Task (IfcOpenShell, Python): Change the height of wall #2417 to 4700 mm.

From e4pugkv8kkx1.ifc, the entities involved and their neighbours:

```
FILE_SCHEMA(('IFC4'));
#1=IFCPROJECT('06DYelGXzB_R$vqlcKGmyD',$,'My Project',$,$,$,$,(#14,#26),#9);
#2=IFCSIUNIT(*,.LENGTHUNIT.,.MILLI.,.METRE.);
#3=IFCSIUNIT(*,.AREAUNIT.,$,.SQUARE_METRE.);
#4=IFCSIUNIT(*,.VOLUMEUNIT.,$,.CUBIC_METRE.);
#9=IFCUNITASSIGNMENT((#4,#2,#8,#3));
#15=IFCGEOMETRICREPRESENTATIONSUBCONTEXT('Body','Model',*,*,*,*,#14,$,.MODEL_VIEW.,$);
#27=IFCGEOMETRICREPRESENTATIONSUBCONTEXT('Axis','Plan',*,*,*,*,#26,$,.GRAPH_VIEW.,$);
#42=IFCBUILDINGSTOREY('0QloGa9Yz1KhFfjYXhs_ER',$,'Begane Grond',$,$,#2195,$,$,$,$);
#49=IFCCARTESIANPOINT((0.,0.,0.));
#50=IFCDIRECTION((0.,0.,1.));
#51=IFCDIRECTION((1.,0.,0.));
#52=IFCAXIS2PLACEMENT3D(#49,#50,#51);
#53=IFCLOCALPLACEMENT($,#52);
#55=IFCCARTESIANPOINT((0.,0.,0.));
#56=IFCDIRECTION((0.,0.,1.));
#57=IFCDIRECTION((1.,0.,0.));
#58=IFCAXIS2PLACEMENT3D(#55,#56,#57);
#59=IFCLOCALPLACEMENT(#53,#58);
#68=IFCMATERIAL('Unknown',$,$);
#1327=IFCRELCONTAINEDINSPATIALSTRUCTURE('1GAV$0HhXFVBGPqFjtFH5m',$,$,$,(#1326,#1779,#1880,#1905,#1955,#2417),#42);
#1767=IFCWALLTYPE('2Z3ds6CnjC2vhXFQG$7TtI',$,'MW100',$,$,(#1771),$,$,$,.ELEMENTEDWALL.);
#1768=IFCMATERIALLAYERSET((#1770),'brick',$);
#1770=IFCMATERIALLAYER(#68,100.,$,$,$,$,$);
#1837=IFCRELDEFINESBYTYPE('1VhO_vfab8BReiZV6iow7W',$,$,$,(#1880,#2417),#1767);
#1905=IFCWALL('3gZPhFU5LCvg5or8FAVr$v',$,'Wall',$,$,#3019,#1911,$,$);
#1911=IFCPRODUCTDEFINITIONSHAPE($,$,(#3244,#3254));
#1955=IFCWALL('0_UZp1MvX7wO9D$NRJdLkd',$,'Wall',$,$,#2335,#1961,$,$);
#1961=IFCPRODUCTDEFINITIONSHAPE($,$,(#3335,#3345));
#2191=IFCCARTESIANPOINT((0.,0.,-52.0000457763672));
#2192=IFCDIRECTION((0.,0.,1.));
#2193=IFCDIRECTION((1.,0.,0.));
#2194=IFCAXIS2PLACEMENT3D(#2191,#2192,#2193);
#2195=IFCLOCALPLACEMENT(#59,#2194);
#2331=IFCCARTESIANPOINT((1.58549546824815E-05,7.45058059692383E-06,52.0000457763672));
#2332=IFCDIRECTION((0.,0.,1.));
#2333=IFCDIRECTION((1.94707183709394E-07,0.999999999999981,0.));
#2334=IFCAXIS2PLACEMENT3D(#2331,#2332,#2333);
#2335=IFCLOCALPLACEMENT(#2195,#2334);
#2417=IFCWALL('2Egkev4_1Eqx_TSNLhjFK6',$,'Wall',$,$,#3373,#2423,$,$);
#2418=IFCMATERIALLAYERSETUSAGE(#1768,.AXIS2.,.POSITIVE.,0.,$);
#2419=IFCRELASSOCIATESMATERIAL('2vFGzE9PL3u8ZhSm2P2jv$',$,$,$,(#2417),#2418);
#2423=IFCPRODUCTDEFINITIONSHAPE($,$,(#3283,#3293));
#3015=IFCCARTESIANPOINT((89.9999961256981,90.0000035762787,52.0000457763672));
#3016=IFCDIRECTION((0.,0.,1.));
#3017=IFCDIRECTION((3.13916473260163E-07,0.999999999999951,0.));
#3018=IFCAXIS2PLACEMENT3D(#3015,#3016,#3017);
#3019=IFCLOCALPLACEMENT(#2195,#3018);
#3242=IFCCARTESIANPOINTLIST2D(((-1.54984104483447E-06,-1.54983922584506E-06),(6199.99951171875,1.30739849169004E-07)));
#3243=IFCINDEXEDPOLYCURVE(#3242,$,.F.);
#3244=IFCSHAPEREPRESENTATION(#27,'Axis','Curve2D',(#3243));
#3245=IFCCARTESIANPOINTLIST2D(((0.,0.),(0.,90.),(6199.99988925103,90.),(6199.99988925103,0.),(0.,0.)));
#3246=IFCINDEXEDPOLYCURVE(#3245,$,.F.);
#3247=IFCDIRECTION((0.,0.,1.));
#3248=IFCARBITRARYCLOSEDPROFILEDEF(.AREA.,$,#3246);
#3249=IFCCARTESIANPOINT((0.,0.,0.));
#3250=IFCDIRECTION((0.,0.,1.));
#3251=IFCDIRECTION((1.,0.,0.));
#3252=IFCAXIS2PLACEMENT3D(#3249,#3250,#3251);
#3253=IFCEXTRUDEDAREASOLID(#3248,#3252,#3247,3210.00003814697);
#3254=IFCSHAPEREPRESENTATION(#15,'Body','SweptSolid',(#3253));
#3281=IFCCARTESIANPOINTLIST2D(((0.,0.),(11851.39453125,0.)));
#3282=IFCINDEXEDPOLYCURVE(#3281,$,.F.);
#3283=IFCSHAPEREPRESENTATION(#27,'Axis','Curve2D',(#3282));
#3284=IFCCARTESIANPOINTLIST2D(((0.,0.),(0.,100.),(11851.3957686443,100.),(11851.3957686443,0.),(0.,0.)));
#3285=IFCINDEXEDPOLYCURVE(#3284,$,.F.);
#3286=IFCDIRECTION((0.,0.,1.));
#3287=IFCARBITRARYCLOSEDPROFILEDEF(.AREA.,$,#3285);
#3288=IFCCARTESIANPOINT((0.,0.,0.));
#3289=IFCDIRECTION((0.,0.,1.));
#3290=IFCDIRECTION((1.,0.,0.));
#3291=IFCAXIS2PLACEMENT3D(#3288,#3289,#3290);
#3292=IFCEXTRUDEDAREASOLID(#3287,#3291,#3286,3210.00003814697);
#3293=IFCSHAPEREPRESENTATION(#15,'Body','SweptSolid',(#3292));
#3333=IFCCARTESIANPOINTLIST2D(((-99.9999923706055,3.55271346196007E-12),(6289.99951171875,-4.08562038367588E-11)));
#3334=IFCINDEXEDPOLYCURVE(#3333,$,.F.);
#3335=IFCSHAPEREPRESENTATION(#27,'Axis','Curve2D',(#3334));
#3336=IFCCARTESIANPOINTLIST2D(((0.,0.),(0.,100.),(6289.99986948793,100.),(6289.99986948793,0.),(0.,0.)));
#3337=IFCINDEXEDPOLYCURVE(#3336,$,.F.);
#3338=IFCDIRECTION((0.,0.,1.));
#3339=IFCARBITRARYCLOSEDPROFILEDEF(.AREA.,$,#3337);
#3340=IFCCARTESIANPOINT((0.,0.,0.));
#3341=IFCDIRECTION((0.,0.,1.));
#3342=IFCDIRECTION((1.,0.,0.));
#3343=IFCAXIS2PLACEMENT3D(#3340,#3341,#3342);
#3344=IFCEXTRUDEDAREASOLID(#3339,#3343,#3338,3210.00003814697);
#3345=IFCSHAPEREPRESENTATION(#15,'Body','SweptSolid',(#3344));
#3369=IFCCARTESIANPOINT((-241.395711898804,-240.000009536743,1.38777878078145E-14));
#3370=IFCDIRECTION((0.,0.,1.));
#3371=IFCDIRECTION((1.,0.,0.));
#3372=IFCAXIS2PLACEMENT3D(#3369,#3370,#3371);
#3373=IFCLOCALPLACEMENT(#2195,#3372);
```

```python
import ifcopenshell
import ifcopenshell.geom
import ifcopenshell.util.representation
import ifcopenshell.util.shape
import ifcopenshell.util.unit

model = ifcopenshell.open("e4pugkv8kkx1.ifc")
unit_scale = ifcopenshell.util.unit.calculate_unit_scale(model)
settings = ifcopenshell.geom.settings()


def volume(element):
    """Net volume in cubic metres, openings subtracted."""
    shape = ifcopenshell.geom.create_shape(settings, element)
    return ifcopenshell.util.shape.get_volume(shape.geometry)


wall = model.by_id(2417)
before = volume(wall)

body = ifcopenshell.util.representation.get_representation(wall, "Model", "Body")
solid = body.Items[0]
old_height = solid.Depth
solid.Depth = 4.7 / unit_scale
after = volume(wall)

print(f"height {old_height:g} -> {solid.Depth:g}, volume {before:.3f} -> {after:.3f} m3")

model.write("e4pugkv8kkx1_updated.ifc")
```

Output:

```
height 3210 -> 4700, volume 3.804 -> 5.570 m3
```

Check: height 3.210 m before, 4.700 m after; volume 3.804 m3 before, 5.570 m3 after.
